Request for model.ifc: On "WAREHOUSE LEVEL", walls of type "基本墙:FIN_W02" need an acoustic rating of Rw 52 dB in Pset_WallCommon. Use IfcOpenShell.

First a look at what the model holds.

```python
import ifcopenshell
import ifcopenshell.util.element

model = ifcopenshell.open("model.ifc")
print(model.schema)
storey = next(s for s in model.by_type("IfcBuildingStorey") if s.Name == "WAREHOUSE LEVEL")
walls = [e for e in ifcopenshell.util.element.get_decomposition(storey) if e.is_a("IfcWall")]
seen = {}
for e in walls:
    element_type = ifcopenshell.util.element.get_type(e)
    key = (element_type.Name if element_type != e and element_type else None, ifcopenshell.util.element.get_pset(e, "Pset_WallCommon", "AcousticRating"))
    seen[key] = seen.get(key, 0) + 1
for (name, value), count in sorted(seen.items(), key=str):
    print(count, "x", name, "|", value)
```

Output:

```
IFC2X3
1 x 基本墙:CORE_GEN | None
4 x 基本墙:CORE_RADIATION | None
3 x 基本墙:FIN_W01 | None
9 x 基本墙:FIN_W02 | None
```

```python
import ifcopenshell
import ifcopenshell.api.pset
import ifcopenshell.util.element

model = ifcopenshell.open("model.ifc")

storey = next(s for s in model.by_type("IfcBuildingStorey") if s.Name == "WAREHOUSE LEVEL")
walls = [e for e in ifcopenshell.util.element.get_decomposition(storey) if e.is_a("IfcWall")]

count = 0
for e in walls:
    element_type = ifcopenshell.util.element.get_type(e)
    if element_type in (None, e) or element_type.Name != "基本墙:FIN_W02":
        continue
    # add_pset returns the element's existing set when there is one.
    pset = ifcopenshell.api.pset.add_pset(model, product=e, name="Pset_WallCommon")
    ifcopenshell.api.pset.edit_pset(model, pset=pset, properties={"AcousticRating": "Rw 52 dB"})
    count += 1

print(count, "walls updated")

model.write("model_updated.ifc")
```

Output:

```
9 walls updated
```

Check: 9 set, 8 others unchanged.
